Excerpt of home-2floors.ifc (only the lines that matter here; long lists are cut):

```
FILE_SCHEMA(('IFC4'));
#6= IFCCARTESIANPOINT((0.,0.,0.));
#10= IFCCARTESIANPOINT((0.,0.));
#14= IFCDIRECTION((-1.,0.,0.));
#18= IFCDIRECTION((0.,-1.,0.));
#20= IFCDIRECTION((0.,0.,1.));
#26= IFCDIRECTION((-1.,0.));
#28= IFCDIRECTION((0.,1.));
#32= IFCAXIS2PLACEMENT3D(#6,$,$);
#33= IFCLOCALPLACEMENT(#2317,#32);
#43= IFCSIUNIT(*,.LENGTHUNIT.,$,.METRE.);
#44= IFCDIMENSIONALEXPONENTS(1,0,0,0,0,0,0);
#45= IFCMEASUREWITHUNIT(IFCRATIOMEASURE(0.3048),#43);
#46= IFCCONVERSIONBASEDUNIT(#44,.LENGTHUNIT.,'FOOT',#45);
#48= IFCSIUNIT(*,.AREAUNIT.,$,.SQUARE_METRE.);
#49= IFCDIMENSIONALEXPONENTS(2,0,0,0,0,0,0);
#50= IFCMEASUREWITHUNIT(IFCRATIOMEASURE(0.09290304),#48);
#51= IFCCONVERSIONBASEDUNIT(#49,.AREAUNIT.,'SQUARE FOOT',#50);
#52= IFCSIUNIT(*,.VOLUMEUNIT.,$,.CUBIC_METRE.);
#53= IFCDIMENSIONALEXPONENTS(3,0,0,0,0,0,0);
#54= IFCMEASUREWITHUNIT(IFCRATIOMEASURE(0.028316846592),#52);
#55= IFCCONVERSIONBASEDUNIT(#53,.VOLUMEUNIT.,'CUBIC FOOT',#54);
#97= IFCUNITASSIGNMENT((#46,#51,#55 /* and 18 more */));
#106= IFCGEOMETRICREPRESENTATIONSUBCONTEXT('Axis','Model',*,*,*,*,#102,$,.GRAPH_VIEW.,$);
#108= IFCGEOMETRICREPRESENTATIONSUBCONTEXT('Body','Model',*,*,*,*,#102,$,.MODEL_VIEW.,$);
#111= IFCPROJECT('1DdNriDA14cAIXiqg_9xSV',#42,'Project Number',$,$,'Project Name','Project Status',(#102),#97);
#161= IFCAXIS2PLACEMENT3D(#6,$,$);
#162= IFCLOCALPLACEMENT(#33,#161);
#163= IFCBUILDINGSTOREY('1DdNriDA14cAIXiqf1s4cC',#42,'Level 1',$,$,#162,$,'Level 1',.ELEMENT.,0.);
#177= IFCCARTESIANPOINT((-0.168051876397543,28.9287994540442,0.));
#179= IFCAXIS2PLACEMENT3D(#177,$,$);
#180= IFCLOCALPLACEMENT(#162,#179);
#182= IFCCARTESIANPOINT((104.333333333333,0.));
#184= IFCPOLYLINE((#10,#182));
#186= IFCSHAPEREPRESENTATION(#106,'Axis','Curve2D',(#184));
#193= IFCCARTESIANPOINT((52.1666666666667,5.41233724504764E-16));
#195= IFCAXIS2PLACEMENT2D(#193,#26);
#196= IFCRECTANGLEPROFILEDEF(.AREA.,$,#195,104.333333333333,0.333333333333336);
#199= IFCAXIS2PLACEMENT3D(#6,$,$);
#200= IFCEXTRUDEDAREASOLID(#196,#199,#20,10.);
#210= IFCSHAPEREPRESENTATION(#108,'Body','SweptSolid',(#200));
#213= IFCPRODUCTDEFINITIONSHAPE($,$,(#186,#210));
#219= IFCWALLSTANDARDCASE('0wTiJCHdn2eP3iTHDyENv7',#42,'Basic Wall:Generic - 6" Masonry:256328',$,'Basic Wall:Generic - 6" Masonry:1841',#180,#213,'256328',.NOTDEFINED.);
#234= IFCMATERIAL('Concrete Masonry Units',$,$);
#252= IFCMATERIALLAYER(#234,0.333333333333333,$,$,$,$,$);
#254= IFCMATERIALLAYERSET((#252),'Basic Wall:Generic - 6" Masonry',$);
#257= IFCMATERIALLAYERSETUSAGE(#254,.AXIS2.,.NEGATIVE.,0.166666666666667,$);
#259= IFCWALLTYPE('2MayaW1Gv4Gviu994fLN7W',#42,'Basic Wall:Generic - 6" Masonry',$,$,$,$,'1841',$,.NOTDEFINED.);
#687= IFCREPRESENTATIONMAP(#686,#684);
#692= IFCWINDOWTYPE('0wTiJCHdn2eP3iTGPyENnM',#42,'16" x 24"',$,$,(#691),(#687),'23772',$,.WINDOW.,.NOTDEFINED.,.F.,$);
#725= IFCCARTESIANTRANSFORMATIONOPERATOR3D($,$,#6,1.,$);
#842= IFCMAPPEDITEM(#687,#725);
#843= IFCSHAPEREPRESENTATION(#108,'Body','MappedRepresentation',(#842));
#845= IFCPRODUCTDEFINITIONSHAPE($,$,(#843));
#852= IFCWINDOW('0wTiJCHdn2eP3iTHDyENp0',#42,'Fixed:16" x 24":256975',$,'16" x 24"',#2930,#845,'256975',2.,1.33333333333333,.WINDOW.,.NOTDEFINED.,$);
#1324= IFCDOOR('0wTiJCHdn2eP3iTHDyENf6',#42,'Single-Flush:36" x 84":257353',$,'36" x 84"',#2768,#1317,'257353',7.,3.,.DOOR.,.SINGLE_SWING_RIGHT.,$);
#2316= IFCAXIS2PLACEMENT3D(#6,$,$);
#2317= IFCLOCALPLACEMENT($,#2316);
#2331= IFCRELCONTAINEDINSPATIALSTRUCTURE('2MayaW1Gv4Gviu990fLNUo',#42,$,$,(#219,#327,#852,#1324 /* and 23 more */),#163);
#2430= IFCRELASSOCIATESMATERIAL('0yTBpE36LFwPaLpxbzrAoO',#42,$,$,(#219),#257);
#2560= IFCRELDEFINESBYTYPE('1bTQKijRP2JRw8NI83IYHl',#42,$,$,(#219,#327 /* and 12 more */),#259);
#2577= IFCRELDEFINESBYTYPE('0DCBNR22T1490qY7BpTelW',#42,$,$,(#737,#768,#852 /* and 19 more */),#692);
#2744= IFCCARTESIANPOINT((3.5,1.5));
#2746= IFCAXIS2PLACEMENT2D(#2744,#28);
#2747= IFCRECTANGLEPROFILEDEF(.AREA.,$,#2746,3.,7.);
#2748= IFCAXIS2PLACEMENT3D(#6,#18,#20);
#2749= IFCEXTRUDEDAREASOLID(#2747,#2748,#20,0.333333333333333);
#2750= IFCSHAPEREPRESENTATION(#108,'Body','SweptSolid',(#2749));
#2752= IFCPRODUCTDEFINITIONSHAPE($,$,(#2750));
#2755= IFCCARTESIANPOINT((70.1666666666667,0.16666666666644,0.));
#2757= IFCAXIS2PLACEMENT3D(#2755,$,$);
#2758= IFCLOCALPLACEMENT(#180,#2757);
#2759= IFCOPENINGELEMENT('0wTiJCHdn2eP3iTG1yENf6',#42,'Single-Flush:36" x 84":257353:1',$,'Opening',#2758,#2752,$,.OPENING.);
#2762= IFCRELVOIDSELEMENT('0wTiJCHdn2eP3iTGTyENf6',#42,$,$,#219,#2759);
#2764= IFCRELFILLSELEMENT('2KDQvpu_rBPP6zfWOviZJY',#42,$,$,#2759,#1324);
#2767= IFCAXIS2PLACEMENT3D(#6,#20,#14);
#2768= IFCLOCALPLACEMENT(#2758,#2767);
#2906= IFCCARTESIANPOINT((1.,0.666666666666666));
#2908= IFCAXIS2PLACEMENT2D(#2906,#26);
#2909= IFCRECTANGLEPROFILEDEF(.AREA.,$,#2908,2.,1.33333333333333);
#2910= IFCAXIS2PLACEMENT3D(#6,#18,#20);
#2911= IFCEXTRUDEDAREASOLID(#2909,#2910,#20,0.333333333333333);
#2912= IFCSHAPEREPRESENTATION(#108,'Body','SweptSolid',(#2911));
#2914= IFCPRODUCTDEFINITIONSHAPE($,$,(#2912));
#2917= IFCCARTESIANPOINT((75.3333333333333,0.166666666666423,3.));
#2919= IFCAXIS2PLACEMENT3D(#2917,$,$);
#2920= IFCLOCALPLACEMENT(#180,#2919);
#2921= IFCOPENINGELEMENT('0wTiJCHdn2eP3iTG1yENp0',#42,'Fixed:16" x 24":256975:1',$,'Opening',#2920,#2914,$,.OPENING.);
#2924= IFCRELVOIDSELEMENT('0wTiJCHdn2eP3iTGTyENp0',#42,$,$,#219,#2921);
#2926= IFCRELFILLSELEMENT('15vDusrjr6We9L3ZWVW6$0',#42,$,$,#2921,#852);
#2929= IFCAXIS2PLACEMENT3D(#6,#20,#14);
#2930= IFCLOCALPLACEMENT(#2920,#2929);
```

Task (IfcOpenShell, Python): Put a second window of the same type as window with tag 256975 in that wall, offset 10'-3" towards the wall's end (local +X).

```python
import ifcopenshell
import ifcopenshell.api.feature
import ifcopenshell.api.geometry
import ifcopenshell.api.root
import ifcopenshell.geom
import ifcopenshell.util.element
import ifcopenshell.util.placement
import ifcopenshell.util.shape
import ifcopenshell.util.unit

model = ifcopenshell.open("home-2floors.ifc")
unit_scale = ifcopenshell.util.unit.calculate_unit_scale(model)
settings = ifcopenshell.geom.settings()


def volume(element):
    """Net volume in cubic metres, openings subtracted."""
    shape = ifcopenshell.geom.create_shape(settings, element)
    return ifcopenshell.util.shape.get_volume(shape.geometry)


def reuse_history(source, copy):
    """copy_class also copies each property set's owner history, people and application; keep the originals."""
    for rel in copy.IsDefinedBy:
        if rel.is_a("IfcRelDefinesByProperties") and (history := rel.RelatingPropertyDefinition.OwnerHistory):
            rel.RelatingPropertyDefinition.OwnerHistory = source.OwnerHistory
            ifcopenshell.util.element.remove_deep2(model, history)


window = model.by_guid("0wTiJCHdn2eP3iTHDyENp0")
opening = window.FillsVoids[0].RelatingOpeningElement
wall = opening.VoidsElements[0].RelatingBuildingElement
before = volume(wall)
shift = ifcopenshell.util.placement.get_local_placement(wall.ObjectPlacement)[:3, 0] * 123 * 0.0254 / unit_scale

# copy_class copies the void relationship, type, container and properties, but no geometry.
new_opening = ifcopenshell.api.root.copy_class(model, product=opening)
new_opening.Representation = ifcopenshell.util.element.copy_deep(
    model, opening.Representation, exclude=["IfcGeometricRepresentationContext", "IfcRepresentationMap"]
)
new_opening.Name = 'Fixed:16" x 24"'
new_window = ifcopenshell.api.root.copy_class(model, product=window)
new_window.Representation = ifcopenshell.util.element.copy_deep(
    model, window.Representation, exclude=["IfcGeometricRepresentationContext", "IfcRepresentationMap"]
)
new_window.Name = 'Fixed:16" x 24"'
new_window.Tag = None
reuse_history(window, new_window)
ifcopenshell.api.feature.add_filling(model, opening=new_opening, element=new_window)

for old, new in ((opening, new_opening), (window, new_window)):
    matrix = ifcopenshell.util.placement.get_local_placement(old.ObjectPlacement)
    matrix[:3, 3] += shift
    ifcopenshell.api.geometry.edit_object_placement(model, product=new, matrix=matrix, is_si=False)

after = volume(wall)

print(f"wall volume {before:.3f} -> {after:.3f} m3")

model.write("home-2floors_rev.ifc")
```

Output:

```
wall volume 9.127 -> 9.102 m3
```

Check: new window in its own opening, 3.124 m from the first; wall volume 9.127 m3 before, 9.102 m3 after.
